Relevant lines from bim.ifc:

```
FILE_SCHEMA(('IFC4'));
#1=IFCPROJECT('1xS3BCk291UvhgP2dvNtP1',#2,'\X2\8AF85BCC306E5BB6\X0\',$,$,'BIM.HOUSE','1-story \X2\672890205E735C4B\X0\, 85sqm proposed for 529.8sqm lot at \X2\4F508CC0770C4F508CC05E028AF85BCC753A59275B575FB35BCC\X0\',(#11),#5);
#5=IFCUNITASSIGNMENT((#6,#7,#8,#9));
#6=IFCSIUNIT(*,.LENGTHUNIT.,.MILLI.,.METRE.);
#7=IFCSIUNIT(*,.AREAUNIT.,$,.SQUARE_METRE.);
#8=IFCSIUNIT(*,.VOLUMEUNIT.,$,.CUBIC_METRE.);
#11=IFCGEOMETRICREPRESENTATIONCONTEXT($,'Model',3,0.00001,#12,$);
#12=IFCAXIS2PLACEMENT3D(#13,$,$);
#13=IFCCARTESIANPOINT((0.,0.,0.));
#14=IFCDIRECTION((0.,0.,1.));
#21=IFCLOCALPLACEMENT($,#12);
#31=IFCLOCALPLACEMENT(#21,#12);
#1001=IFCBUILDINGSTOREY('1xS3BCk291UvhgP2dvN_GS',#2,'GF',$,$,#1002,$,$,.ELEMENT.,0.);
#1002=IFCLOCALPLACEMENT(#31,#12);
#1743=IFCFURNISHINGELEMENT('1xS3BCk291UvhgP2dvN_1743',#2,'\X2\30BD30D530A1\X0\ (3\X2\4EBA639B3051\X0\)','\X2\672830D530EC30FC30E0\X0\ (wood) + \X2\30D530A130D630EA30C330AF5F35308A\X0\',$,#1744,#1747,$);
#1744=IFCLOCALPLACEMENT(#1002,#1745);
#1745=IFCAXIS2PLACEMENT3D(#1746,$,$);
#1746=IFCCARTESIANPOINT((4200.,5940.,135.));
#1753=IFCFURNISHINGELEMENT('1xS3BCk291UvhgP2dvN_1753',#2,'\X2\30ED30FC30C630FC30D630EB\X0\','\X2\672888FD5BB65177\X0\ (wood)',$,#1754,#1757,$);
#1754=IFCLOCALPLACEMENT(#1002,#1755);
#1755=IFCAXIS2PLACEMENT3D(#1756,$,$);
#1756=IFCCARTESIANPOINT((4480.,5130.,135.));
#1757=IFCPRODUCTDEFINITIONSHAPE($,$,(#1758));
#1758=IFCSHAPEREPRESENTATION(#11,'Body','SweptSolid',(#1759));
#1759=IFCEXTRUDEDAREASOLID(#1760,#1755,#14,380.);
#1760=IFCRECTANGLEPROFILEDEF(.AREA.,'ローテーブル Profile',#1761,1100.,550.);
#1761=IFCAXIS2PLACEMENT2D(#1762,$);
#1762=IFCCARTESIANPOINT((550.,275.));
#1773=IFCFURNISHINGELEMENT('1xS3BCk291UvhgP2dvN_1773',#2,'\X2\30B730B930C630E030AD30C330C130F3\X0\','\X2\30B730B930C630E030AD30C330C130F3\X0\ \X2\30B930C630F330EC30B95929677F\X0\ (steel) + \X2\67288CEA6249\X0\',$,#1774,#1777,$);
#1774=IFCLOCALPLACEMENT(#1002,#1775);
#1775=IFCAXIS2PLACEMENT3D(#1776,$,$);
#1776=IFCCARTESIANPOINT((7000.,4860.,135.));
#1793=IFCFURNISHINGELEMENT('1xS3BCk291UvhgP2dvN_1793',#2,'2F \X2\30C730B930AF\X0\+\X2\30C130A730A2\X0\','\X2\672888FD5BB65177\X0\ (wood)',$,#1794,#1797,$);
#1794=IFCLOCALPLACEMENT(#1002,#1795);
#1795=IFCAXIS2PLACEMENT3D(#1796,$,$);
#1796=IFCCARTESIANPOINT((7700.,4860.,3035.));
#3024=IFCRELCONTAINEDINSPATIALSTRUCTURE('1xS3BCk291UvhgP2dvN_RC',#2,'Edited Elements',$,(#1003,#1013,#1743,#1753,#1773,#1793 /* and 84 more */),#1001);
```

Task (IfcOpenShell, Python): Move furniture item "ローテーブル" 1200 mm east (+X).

```python
import ifcopenshell
import ifcopenshell.api.geometry
import ifcopenshell.util.placement
import ifcopenshell.util.unit

model = ifcopenshell.open("bim.ifc")
unit_scale = ifcopenshell.util.unit.calculate_unit_scale(model)

item = model.by_guid("1xS3BCk291UvhgP2dvN_1753")
matrix = ifcopenshell.util.placement.get_local_placement(item.ObjectPlacement)
matrix[0, 3] += 1.2 / unit_scale
ifcopenshell.api.geometry.edit_object_placement(model, product=item, matrix=matrix, is_si=False)

print(ifcopenshell.util.placement.get_local_placement(item.ObjectPlacement).round(3) + 0.0)

model.write("bim_updated.ifc")
```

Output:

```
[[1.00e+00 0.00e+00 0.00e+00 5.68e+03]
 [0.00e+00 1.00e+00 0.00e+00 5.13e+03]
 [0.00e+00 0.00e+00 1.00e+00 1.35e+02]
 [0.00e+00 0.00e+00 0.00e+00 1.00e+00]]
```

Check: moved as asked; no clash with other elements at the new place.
